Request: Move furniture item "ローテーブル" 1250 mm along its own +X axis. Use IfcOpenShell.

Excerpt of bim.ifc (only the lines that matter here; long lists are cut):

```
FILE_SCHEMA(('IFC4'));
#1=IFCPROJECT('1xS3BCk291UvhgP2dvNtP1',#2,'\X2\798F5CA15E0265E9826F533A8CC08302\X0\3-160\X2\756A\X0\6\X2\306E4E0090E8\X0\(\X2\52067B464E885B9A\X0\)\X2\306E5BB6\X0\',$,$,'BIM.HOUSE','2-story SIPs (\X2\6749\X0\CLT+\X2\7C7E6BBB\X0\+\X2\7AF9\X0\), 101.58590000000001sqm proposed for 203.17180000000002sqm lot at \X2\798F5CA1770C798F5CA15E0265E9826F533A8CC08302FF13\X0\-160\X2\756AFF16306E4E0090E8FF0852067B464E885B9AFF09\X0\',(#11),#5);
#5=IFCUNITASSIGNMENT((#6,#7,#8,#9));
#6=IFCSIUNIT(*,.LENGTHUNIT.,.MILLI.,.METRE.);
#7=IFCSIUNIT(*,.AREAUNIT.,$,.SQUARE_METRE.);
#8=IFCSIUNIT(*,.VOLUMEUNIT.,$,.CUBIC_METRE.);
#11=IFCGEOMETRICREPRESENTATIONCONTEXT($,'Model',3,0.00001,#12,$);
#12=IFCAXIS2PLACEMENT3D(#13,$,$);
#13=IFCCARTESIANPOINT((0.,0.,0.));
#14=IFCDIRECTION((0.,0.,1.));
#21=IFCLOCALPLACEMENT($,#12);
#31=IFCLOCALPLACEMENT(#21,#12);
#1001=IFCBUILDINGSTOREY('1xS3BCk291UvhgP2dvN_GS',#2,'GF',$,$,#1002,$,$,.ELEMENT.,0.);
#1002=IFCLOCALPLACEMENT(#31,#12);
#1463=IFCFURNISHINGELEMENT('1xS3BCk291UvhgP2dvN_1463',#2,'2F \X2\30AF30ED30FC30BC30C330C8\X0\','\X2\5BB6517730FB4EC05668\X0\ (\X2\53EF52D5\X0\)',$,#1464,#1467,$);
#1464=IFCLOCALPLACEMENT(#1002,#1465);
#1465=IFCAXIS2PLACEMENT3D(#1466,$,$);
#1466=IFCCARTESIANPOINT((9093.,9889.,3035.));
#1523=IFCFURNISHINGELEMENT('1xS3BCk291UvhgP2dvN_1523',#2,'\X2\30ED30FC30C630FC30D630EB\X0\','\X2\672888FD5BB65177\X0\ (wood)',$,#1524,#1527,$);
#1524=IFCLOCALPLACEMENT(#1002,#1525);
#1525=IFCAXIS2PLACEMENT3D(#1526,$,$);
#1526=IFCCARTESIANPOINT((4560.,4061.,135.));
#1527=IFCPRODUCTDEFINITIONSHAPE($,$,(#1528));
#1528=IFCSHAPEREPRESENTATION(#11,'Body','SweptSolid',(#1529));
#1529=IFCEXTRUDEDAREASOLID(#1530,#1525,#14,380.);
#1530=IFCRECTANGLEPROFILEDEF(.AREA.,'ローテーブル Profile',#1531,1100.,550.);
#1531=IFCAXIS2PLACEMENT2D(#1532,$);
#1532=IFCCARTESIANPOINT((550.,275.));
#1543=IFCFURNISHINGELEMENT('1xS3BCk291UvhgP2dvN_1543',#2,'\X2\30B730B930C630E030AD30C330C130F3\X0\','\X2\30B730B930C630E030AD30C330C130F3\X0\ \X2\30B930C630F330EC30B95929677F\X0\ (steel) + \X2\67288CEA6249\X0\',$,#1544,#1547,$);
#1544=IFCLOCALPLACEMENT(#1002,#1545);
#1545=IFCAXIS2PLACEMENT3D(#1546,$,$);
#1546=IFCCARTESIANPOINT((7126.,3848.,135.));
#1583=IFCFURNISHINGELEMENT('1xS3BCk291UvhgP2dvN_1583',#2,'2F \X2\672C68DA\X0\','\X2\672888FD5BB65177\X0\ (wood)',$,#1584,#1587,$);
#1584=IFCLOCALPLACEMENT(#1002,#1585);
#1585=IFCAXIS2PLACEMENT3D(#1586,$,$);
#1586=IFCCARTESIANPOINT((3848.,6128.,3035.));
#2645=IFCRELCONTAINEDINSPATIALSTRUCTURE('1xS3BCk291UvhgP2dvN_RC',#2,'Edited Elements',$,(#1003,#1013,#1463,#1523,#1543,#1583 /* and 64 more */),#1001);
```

```python
import ifcopenshell
import ifcopenshell.api.geometry
import ifcopenshell.util.placement

model = ifcopenshell.open("bim.ifc")

item = model.by_id(1523)
matrix = ifcopenshell.util.placement.get_local_placement(item.ObjectPlacement)
matrix[:3, 3] += matrix[:3, 0] * 1250.0
ifcopenshell.api.geometry.edit_object_placement(model, product=item, matrix=matrix, is_si=False)

print(ifcopenshell.util.placement.get_local_placement(item.ObjectPlacement).round(3) + 0.0)

model.write("bim-out.ifc")
```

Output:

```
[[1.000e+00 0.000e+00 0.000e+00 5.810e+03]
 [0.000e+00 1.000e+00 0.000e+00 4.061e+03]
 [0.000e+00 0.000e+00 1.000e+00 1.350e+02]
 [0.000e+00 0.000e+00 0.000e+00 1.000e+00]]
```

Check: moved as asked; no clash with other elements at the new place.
